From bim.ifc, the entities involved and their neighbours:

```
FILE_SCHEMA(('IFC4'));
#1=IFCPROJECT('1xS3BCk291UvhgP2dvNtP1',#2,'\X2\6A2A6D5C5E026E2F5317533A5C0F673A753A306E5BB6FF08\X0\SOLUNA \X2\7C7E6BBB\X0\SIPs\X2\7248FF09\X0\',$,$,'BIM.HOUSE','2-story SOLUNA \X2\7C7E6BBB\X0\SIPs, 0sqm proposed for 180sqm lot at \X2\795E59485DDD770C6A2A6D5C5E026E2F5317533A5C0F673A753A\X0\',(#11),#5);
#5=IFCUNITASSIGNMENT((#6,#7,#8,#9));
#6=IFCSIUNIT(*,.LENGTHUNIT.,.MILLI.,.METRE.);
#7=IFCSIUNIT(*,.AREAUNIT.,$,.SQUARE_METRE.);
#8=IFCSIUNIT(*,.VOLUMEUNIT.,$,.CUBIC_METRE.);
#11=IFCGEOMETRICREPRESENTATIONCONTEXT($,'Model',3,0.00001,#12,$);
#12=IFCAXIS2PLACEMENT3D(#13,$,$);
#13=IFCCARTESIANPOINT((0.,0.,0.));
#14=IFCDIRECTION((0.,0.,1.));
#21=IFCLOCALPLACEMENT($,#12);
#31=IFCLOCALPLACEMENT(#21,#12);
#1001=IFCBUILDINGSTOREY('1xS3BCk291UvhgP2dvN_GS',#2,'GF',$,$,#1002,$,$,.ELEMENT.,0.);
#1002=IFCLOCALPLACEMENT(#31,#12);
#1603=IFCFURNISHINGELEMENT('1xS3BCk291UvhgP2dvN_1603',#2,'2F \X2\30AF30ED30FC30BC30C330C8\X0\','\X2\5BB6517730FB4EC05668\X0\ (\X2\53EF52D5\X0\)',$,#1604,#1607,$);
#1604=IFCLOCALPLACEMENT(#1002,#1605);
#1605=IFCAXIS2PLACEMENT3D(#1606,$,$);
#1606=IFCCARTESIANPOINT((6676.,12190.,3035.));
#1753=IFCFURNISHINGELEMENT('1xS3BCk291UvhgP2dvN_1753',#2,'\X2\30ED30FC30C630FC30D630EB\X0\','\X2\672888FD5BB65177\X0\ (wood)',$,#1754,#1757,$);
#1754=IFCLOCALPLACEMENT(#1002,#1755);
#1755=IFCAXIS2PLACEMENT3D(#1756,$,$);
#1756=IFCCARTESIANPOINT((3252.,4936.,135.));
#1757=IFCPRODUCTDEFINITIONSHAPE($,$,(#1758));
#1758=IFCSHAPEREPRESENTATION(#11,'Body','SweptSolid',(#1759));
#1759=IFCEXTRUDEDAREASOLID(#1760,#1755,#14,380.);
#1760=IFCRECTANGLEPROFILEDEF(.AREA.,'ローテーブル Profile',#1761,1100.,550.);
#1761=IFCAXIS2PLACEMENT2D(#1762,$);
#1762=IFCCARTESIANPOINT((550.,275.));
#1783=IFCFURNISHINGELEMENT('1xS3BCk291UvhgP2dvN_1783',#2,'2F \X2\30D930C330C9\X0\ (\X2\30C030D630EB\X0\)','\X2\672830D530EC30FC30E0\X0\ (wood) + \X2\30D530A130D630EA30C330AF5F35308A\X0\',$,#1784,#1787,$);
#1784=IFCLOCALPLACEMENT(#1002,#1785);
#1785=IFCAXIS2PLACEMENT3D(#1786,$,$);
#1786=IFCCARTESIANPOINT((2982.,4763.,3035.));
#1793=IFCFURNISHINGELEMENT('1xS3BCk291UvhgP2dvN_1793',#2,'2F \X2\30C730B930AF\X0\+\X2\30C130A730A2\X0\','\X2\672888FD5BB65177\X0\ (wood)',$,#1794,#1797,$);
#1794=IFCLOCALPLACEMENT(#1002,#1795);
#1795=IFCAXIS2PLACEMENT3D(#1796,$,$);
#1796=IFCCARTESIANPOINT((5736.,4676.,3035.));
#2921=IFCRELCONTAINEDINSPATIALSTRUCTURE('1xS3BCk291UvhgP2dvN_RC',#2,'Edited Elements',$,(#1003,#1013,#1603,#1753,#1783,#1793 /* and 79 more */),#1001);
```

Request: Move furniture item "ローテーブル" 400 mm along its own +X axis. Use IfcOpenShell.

```python
import ifcopenshell
import ifcopenshell.api.geometry
import ifcopenshell.util.placement
import ifcopenshell.util.unit

model = ifcopenshell.open("bim.ifc")
unit_scale = ifcopenshell.util.unit.calculate_unit_scale(model)

item = model.by_guid("1xS3BCk291UvhgP2dvN_1753")
matrix = ifcopenshell.util.placement.get_local_placement(item.ObjectPlacement)
matrix[:3, 3] += matrix[:3, 0] * 0.4 / unit_scale
ifcopenshell.api.geometry.edit_object_placement(model, product=item, matrix=matrix, is_si=False)

print(ifcopenshell.util.placement.get_local_placement(item.ObjectPlacement).round(3) + 0.0)

model.write("bim_edited.ifc")
```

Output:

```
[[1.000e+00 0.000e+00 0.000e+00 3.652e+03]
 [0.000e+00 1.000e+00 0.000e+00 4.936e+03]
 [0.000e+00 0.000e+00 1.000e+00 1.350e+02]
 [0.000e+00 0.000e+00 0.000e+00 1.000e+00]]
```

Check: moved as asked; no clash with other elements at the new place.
